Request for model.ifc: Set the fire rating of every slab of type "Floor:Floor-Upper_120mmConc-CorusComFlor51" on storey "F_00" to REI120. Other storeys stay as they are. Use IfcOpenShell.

First a look at what the model holds.

```python
import ifcopenshell
import ifcopenshell.util.element

model = ifcopenshell.open("model.ifc")
print(model.schema)
storey = next(s for s in model.by_type("IfcBuildingStorey") if s.Name == "F_00")
slabs = [e for e in ifcopenshell.util.element.get_decomposition(storey) if e.is_a("IfcSlab")]
seen = {}
for e in slabs:
    element_type = ifcopenshell.util.element.get_type(e)
    key = (element_type.Name if element_type != e and element_type else None, ifcopenshell.util.element.get_pset(e, "Pset_SlabCommon", "FireRating"))
    seen[key] = seen.get(key, 0) + 1
for (name, value), count in sorted(seen.items(), key=str):
    print(count, "x", name, "|", value)
```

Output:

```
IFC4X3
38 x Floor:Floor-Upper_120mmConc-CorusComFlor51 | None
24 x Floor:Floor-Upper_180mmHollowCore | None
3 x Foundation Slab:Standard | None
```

```python
import ifcopenshell
import ifcopenshell.api.pset
import ifcopenshell.util.element

model = ifcopenshell.open("model.ifc")

storey = next(s for s in model.by_type("IfcBuildingStorey") if s.Name == "F_00")
slabs = [e for e in ifcopenshell.util.element.get_decomposition(storey) if e.is_a("IfcSlab")]

count = 0
for e in slabs:
    element_type = ifcopenshell.util.element.get_type(e)
    if element_type in (None, e) or element_type.Name != "Floor:Floor-Upper_120mmConc-CorusComFlor51":
        continue
    # add_pset returns the element's existing set when there is one.
    pset = ifcopenshell.api.pset.add_pset(model, product=e, name="Pset_SlabCommon")
    ifcopenshell.api.pset.edit_pset(model, pset=pset, properties={"FireRating": "REI120"})
    count += 1

print(count, "slabs updated")

model.write("model_v2.ifc")
```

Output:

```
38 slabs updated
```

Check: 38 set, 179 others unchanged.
